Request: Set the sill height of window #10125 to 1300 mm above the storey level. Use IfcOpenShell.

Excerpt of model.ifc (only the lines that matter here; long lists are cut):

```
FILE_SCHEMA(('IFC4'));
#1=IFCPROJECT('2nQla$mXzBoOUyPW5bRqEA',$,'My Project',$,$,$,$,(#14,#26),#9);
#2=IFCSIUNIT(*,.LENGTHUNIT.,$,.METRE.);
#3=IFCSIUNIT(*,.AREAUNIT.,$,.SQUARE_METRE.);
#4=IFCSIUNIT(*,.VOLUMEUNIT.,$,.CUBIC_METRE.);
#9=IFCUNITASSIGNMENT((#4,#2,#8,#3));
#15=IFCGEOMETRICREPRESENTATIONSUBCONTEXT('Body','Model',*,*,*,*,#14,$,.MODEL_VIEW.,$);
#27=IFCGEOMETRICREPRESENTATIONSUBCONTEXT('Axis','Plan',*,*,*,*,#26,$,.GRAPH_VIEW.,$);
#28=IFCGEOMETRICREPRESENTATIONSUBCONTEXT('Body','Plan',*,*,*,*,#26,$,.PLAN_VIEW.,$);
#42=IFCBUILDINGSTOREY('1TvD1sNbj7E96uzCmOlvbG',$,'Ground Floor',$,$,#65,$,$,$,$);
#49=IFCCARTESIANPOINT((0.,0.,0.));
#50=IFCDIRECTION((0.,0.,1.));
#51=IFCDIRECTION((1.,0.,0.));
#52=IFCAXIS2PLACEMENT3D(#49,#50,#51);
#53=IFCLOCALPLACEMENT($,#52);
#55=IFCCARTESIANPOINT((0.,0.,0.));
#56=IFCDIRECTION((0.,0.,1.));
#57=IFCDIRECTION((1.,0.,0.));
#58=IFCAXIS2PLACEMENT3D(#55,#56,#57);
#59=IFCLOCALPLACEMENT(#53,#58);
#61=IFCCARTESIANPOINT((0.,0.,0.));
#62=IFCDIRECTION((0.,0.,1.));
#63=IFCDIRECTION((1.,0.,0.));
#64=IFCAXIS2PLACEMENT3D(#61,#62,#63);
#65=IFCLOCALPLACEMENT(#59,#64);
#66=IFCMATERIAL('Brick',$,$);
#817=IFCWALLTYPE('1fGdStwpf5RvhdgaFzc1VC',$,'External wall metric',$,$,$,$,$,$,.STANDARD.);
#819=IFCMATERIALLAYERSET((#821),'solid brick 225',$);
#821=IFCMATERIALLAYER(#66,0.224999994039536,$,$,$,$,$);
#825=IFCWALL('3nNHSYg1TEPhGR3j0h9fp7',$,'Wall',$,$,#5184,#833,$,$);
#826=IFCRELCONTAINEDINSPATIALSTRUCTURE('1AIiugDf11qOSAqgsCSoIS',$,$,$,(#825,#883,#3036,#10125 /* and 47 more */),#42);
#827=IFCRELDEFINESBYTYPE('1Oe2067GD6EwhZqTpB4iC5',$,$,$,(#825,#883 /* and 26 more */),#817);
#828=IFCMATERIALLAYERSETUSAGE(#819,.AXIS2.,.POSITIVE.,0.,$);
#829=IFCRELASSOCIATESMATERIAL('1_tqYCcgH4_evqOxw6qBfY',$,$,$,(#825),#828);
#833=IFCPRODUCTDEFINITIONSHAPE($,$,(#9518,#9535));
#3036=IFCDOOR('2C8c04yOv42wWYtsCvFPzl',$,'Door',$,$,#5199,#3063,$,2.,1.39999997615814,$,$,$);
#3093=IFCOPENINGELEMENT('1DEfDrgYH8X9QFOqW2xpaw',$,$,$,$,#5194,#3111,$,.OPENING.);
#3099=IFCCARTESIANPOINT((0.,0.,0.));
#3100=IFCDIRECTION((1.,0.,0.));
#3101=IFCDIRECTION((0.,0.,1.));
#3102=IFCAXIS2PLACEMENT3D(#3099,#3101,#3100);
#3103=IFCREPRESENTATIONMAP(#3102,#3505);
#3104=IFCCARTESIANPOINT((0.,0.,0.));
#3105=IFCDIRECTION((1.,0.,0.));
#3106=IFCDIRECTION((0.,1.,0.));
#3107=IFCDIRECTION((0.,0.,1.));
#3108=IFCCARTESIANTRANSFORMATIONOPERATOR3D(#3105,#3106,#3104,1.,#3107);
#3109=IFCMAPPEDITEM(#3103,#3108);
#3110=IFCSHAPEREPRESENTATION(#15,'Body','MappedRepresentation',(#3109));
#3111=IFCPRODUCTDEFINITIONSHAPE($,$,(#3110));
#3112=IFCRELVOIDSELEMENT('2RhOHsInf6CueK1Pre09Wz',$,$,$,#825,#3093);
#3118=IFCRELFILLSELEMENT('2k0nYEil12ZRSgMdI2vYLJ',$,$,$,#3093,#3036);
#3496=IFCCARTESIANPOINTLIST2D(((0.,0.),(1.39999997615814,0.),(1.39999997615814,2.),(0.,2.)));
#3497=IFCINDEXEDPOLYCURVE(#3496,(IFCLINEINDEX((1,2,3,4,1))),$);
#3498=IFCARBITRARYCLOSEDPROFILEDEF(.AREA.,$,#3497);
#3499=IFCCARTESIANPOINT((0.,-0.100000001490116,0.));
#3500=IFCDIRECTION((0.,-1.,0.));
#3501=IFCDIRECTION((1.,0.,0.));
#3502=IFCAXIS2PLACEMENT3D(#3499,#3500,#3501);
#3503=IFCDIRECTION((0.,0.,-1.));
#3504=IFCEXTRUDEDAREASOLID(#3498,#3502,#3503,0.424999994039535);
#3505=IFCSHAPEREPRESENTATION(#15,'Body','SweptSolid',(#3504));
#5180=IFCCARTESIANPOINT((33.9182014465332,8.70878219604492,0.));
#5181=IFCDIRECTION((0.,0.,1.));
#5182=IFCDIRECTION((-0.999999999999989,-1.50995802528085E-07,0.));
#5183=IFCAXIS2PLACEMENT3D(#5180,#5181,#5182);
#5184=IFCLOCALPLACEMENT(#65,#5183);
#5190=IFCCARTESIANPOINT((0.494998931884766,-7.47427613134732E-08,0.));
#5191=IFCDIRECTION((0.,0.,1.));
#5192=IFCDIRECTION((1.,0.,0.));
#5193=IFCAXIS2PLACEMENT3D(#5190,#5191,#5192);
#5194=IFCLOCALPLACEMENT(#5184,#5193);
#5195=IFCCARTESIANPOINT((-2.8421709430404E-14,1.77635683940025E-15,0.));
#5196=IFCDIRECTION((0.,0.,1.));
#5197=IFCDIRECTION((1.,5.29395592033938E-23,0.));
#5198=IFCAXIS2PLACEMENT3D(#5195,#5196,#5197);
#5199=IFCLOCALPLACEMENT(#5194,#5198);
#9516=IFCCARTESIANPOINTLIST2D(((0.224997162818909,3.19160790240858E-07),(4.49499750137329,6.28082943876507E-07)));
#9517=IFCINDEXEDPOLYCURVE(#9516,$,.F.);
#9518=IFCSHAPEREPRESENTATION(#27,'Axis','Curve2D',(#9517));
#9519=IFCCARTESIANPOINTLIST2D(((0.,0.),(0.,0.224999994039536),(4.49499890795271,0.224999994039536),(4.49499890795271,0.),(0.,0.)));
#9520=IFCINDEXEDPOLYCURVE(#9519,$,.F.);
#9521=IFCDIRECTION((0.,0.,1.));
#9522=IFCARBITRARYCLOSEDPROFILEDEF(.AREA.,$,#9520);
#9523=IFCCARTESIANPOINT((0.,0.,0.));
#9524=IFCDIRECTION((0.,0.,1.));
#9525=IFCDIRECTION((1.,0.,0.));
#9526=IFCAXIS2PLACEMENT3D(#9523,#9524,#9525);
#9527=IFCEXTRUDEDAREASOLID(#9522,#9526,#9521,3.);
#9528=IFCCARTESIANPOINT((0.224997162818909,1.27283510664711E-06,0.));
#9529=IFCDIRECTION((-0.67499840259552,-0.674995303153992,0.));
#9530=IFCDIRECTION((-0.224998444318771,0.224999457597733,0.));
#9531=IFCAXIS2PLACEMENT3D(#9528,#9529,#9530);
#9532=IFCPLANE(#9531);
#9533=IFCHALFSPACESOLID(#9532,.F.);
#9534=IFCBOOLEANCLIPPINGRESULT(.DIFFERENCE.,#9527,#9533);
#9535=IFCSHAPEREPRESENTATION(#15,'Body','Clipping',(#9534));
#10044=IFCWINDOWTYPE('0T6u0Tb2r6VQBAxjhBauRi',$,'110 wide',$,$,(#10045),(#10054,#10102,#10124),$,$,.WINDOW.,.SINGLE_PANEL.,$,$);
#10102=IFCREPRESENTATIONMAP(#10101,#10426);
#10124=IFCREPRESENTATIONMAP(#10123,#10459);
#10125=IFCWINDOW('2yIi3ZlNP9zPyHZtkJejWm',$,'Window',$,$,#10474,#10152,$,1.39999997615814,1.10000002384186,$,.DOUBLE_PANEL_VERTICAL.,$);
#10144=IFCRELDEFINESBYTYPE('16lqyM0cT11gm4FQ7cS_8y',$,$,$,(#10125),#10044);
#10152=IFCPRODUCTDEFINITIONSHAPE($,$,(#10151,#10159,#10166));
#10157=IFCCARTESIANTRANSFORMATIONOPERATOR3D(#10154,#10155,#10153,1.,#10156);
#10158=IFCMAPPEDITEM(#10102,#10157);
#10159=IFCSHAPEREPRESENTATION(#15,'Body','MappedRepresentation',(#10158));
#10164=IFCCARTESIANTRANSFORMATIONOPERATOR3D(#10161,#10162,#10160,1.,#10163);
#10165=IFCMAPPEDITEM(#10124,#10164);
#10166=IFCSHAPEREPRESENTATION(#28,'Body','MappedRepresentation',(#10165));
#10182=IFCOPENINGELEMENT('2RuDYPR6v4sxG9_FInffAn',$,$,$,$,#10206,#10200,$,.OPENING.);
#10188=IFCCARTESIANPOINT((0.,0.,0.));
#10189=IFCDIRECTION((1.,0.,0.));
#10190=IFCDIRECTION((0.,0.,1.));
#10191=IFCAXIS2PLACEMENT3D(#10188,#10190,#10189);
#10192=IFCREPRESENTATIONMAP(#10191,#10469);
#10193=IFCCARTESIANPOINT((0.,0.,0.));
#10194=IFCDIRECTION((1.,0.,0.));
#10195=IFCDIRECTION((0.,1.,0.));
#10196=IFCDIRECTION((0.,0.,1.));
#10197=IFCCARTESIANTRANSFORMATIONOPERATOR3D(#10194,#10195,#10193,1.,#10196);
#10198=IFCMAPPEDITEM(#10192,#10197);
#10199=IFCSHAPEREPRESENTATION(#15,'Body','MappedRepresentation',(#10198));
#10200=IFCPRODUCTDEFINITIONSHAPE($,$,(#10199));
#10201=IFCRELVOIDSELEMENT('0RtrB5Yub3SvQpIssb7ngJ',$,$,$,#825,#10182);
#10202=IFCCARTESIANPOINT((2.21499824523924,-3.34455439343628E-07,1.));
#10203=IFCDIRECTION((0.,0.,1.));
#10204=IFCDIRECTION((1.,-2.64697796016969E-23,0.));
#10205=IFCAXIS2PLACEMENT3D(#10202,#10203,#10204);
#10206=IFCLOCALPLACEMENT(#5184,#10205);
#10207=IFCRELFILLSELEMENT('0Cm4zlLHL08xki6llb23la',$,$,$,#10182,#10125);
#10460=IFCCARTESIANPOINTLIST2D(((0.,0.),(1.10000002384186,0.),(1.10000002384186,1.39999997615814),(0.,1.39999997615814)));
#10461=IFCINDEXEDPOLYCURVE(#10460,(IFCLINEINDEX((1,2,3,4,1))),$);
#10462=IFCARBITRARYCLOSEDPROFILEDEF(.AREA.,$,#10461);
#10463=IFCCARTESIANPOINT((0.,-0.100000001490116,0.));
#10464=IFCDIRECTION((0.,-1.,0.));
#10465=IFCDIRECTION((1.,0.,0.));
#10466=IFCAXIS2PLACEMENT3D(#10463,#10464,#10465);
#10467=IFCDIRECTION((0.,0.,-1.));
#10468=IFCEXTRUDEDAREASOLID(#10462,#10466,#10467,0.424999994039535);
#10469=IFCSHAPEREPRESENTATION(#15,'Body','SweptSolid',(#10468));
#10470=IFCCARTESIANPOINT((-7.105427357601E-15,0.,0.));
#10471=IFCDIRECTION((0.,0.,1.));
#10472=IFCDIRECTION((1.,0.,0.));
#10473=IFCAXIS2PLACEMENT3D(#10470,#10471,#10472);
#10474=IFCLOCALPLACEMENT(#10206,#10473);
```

```python
import numpy as np
import ifcopenshell
import ifcopenshell.api.geometry
import ifcopenshell.geom
import ifcopenshell.util.element
import ifcopenshell.util.placement
import ifcopenshell.util.shape
import ifcopenshell.util.unit

model = ifcopenshell.open("model.ifc")
unit_scale = ifcopenshell.util.unit.calculate_unit_scale(model)

window = model.by_guid("2yIi3ZlNP9zPyHZtkJejWm")
opening = window.FillsVoids[0].RelatingOpeningElement
storey = ifcopenshell.util.element.get_container(window, ifc_class="IfcBuildingStorey")
level = ifcopenshell.util.placement.get_local_placement(storey.ObjectPlacement)[2, 3]

# The opening's origin need not be at the sill, so measure its lowest point.
shape = ifcopenshell.geom.create_shape(ifcopenshell.geom.settings(), opening)
bottom = ifcopenshell.util.shape.get_shape_bottom_elevation(shape, shape.geometry) / unit_scale
dz = level + 1.3 - bottom

shift = np.array([0.0, 0.0, dz])
# The window is placed relative to its opening, so it follows when the opening moves.
matrix = ifcopenshell.util.placement.get_local_placement(opening.ObjectPlacement)
matrix[:3, 3] += shift
ifcopenshell.api.geometry.edit_object_placement(
    model, product=opening, matrix=matrix, is_si=False, should_transform_children=True
)

print(f"moved by {dz * unit_scale:+.3f} m")

model.write("model_rev.ifc")
```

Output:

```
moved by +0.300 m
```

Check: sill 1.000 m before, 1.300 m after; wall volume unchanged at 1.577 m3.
